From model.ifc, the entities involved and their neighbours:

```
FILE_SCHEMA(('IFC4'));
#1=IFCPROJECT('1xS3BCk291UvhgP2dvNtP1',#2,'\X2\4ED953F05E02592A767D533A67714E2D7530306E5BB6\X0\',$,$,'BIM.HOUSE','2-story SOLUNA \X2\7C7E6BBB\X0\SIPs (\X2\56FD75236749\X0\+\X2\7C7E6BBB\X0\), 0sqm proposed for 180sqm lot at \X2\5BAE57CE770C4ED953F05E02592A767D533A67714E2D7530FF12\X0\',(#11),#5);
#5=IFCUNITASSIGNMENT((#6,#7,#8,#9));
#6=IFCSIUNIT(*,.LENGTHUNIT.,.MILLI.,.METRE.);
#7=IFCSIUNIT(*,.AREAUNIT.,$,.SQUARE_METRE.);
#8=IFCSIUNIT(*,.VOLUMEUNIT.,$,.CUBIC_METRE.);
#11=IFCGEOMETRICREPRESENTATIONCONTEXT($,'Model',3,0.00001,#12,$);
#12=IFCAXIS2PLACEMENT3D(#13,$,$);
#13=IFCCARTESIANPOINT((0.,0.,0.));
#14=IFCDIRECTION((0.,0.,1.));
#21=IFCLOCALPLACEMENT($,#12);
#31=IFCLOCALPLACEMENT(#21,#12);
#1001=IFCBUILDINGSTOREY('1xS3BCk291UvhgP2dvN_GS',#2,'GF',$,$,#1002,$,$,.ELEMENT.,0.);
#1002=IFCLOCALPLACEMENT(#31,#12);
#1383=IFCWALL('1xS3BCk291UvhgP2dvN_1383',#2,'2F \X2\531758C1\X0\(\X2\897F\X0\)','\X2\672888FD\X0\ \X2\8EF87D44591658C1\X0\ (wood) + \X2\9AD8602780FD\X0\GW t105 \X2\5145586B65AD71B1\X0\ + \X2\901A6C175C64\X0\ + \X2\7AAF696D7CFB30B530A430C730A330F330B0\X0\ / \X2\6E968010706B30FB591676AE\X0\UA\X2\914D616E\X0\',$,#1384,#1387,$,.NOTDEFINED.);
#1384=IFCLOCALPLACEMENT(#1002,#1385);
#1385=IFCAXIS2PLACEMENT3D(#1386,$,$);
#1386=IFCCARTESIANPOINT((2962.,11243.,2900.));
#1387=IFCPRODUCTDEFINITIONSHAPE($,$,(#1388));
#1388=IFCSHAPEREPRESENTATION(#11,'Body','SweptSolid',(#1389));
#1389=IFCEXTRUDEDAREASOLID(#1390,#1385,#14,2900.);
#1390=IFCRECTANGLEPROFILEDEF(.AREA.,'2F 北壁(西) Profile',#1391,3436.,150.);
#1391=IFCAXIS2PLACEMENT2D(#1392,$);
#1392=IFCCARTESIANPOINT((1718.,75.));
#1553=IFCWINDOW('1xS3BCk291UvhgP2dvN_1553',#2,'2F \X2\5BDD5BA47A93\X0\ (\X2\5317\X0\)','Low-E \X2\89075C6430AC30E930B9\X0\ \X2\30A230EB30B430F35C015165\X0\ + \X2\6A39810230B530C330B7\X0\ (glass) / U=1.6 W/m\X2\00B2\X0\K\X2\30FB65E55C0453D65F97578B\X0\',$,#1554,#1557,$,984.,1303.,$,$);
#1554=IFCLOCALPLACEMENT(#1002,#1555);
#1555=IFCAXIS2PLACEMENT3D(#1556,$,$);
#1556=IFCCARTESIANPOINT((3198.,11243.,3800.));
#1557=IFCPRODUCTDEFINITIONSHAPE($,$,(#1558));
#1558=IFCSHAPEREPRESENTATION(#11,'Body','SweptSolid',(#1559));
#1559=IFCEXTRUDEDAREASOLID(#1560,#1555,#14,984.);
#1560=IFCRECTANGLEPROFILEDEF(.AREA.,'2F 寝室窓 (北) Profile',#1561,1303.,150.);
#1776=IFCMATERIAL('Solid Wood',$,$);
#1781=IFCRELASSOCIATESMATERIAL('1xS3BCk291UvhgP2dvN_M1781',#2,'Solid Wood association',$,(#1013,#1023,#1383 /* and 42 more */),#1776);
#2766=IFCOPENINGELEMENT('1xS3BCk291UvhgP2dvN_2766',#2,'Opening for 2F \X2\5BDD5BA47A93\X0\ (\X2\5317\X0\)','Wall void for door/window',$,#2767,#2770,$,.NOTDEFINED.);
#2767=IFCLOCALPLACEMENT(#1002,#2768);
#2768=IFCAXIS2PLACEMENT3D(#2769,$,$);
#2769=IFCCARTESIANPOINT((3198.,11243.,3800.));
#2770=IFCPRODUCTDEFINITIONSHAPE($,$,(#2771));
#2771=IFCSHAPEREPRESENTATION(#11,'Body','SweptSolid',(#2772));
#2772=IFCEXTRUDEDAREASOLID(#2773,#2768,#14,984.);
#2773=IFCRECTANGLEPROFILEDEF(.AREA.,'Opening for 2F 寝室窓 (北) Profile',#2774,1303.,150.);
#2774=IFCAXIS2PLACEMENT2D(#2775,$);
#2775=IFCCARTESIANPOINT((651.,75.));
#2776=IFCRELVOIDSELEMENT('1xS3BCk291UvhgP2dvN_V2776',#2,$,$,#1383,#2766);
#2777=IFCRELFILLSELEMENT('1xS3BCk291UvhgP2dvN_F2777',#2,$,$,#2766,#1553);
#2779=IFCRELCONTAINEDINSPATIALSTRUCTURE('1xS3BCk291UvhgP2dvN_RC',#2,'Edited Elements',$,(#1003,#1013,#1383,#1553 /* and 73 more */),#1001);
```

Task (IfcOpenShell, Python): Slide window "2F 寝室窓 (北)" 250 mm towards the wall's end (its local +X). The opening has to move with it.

```python
import ifcopenshell
import ifcopenshell.api.geometry
import ifcopenshell.util.placement
import ifcopenshell.util.unit

model = ifcopenshell.open("model.ifc")
unit_scale = ifcopenshell.util.unit.calculate_unit_scale(model)

window = model.by_id(1553)
opening = window.FillsVoids[0].RelatingOpeningElement
wall = opening.VoidsElements[0].RelatingBuildingElement

wall_matrix = ifcopenshell.util.placement.get_local_placement(wall.ObjectPlacement)
shift = wall_matrix[:3, 0] * 0.25 / unit_scale
before = ifcopenshell.util.placement.get_local_placement(window.ObjectPlacement)[:3, 3].copy()

# The window is not placed relative to its opening, so move both.
for product in (opening, window):
    matrix = ifcopenshell.util.placement.get_local_placement(product.ObjectPlacement)
    matrix[:3, 3] += shift
    ifcopenshell.api.geometry.edit_object_placement(model, product=product, matrix=matrix, is_si=False)

after = ifcopenshell.util.placement.get_local_placement(window.ObjectPlacement)[:3, 3]
print("window moved by", (after - before).round(3) + 0.0)

model.write("model-out.ifc")
```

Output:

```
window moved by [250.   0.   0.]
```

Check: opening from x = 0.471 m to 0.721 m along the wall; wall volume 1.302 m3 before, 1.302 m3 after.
